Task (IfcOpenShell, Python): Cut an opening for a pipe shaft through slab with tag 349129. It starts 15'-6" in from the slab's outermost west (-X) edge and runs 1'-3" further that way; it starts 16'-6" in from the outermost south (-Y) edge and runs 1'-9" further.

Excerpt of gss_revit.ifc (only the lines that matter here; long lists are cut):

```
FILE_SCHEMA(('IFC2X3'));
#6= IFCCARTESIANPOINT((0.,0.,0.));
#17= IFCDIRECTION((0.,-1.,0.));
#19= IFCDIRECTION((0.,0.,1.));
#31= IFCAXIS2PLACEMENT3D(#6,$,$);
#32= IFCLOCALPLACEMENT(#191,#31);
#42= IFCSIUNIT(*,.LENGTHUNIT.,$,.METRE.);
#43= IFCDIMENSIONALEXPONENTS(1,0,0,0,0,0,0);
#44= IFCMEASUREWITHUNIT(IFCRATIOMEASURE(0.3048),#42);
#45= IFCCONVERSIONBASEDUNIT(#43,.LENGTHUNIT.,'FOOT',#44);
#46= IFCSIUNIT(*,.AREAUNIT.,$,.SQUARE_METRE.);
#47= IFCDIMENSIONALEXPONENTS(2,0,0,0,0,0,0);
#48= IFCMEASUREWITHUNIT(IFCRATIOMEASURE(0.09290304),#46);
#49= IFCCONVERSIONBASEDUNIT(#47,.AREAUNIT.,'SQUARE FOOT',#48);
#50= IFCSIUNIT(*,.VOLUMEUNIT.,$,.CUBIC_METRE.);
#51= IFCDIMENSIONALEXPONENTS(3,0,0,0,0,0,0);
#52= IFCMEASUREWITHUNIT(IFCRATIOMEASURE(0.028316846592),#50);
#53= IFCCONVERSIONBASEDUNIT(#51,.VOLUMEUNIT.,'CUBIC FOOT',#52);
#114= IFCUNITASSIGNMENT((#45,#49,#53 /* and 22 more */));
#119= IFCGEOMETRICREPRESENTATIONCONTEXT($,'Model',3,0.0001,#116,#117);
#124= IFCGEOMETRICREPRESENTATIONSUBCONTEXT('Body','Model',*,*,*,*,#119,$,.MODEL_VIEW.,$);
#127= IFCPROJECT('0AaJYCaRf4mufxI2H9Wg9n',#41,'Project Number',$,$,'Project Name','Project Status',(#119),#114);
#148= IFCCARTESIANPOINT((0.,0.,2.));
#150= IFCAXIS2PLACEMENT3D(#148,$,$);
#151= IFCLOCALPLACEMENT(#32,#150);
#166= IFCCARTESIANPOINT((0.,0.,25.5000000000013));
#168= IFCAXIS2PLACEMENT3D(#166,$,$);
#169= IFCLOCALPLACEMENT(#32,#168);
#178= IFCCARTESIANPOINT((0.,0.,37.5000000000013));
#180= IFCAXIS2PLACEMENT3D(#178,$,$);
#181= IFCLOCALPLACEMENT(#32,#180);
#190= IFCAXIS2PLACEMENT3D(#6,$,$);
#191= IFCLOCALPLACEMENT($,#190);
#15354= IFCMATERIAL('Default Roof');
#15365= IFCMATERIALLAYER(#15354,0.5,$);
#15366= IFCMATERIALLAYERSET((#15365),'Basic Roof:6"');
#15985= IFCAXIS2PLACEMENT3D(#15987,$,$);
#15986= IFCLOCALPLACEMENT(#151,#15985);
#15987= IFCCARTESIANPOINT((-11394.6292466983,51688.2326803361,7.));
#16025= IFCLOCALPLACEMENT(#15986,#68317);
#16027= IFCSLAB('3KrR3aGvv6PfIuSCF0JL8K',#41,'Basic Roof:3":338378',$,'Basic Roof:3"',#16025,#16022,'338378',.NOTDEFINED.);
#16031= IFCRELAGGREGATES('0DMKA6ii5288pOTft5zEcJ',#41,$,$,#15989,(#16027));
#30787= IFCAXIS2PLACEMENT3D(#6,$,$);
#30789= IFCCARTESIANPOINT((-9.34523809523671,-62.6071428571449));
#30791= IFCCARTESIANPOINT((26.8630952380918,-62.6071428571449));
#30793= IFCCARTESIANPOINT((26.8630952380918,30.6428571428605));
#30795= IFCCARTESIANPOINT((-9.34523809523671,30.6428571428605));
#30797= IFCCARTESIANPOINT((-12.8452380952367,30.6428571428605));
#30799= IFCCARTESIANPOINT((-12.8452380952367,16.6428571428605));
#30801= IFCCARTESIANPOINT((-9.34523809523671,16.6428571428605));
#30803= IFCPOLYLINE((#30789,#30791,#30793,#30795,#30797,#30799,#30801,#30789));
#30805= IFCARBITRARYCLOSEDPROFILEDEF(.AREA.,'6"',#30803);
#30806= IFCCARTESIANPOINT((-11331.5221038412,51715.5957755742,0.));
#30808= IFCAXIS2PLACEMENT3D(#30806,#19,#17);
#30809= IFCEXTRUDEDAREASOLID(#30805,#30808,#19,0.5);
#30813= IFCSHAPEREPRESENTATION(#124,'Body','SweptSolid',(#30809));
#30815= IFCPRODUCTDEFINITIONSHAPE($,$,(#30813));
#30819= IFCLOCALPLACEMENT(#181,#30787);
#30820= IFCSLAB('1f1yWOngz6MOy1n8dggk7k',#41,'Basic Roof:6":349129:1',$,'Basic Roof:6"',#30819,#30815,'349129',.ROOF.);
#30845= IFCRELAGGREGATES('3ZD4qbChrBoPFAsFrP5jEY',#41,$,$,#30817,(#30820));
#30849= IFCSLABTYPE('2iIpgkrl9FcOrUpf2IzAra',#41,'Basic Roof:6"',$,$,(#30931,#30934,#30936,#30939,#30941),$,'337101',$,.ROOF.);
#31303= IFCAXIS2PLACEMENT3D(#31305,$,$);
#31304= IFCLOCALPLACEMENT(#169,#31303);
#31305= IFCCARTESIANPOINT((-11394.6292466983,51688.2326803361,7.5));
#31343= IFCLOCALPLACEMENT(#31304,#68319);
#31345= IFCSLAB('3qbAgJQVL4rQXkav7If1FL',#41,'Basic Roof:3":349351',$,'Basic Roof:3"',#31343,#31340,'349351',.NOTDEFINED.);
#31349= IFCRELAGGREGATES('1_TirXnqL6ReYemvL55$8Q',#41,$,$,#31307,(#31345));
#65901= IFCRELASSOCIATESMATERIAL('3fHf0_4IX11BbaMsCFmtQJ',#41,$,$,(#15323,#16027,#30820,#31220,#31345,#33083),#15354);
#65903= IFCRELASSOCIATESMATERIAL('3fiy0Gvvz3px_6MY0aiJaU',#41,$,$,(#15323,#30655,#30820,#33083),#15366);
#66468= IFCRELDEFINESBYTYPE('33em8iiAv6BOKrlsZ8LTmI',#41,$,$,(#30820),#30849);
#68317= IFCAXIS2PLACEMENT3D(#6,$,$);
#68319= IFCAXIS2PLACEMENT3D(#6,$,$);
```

```python
import numpy as np
import ifcopenshell
import ifcopenshell.api.feature
import ifcopenshell.api.geometry
import ifcopenshell.api.root
import ifcopenshell.geom
import ifcopenshell.util.placement
import ifcopenshell.util.representation
import ifcopenshell.util.shape
import ifcopenshell.util.unit

model = ifcopenshell.open("gss_revit.ifc")
unit_scale = ifcopenshell.util.unit.calculate_unit_scale(model)
settings = ifcopenshell.geom.settings()


def volume(element):
    """Net volume in cubic metres, openings subtracted."""
    shape = ifcopenshell.geom.create_shape(settings, element)
    return ifcopenshell.util.shape.get_volume(shape.geometry)


slab = model.by_guid("1f1yWOngz6MOy1n8dggk7k")
before = volume(slab)

# Extent in the slab's own axes, in metres. The edges named are its -X and -Y sides.
slab_shape = ifcopenshell.geom.create_shape(settings, slab)
vertices = ifcopenshell.util.shape.get_vertices(slab_shape.geometry)
x_min, y_min, bottom = vertices.min(axis=0)
top = vertices[:, 2].max()

opening = ifcopenshell.api.root.create_entity(model, ifc_class="IfcOpeningElement", name="Pipe shaft opening")
context = ifcopenshell.util.representation.get_context(model, "Model", "Body", "MODEL_VIEW")
width, depth = 0.381, 0.5334
outline = [(0.0, 0.0), (width, 0.0), (width, depth), (0.0, depth), (0.0, 0.0)]
# Overshoot both faces by 50 mm so the cut is clean.
shape = ifcopenshell.api.geometry.add_slab_representation(
    model, context=context, depth=top - bottom + 0.1, polyline=outline
)
ifcopenshell.api.geometry.assign_representation(model, product=opening, representation=shape)

matrix = ifcopenshell.util.placement.get_local_placement(slab.ObjectPlacement)
matrix[:, 3] = matrix @ np.append(np.array([x_min + 4.7244, y_min + 5.0292, bottom - 0.05]) / unit_scale, 1.0)
ifcopenshell.api.geometry.edit_object_placement(model, product=opening, matrix=matrix, is_si=False)
ifcopenshell.api.feature.add_feature(model, feature=opening, element=slab)

after = volume(slab)

print(f"slab volume {before:.3f} -> {after:.3f} m3")

model.write("gss_revit_rev.ifc")
```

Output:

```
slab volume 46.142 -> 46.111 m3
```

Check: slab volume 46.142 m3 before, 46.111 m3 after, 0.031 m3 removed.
